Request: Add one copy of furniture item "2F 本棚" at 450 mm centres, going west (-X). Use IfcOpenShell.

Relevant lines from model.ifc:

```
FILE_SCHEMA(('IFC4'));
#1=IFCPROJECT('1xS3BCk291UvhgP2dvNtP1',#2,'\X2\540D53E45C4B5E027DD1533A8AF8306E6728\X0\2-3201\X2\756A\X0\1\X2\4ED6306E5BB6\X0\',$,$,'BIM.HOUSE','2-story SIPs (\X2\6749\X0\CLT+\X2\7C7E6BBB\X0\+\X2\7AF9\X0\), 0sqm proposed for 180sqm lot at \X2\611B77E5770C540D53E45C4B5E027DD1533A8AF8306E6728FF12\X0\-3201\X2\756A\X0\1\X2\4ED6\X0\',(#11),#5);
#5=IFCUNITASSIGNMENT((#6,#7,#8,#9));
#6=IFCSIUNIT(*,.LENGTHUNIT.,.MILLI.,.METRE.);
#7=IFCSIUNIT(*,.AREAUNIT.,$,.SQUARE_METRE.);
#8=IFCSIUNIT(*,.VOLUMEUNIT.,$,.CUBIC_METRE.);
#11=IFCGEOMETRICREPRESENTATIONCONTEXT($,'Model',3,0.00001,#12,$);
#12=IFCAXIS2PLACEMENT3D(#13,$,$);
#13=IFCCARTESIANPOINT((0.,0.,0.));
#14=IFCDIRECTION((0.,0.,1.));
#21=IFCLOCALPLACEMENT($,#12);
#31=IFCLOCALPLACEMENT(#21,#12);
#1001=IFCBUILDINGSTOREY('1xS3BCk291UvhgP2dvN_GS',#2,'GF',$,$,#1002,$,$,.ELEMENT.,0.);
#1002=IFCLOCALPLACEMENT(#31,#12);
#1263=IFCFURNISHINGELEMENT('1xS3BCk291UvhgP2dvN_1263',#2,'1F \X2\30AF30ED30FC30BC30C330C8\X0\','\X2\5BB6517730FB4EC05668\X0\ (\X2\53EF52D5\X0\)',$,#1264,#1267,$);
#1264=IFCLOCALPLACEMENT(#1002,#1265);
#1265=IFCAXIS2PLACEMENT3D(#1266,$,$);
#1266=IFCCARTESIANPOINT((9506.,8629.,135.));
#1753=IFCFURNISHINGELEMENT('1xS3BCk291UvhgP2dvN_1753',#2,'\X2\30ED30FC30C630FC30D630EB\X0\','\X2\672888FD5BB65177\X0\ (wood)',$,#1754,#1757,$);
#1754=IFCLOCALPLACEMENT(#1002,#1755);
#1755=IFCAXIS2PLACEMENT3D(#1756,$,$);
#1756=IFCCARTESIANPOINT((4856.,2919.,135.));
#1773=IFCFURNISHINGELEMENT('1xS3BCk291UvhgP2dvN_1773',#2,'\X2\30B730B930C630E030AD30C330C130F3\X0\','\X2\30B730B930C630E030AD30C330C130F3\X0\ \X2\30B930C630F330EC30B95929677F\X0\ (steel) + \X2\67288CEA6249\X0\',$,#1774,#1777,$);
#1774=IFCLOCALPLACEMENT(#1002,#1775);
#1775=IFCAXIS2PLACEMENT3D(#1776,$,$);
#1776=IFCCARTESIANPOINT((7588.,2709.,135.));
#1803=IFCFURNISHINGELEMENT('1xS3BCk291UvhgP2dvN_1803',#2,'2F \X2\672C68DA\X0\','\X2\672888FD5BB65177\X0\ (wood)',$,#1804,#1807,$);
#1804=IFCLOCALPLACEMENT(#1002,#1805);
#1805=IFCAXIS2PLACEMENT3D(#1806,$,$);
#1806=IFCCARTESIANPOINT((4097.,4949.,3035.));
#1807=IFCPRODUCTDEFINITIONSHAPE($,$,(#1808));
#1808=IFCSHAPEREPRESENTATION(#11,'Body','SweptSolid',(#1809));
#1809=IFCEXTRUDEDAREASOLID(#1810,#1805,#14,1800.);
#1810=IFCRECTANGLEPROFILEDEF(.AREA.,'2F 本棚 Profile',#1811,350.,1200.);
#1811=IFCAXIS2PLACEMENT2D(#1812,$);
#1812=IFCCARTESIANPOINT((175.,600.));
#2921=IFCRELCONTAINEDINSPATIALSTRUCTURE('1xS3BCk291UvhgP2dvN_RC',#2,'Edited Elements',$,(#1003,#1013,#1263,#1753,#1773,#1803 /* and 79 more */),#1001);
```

```python
import numpy as np
import ifcopenshell
import ifcopenshell.api.geometry
import ifcopenshell.api.root
import ifcopenshell.util.element
import ifcopenshell.util.placement

model = ifcopenshell.open("model.ifc")


def reuse_history(source, copy):
    """copy_class also copies each property set's owner history, people and application; keep the originals."""
    for rel in copy.IsDefinedBy:
        if rel.is_a("IfcRelDefinesByProperties") and (history := rel.RelatingPropertyDefinition.OwnerHistory):
            rel.RelatingPropertyDefinition.OwnerHistory = source.OwnerHistory
            ifcopenshell.util.element.remove_deep2(model, history)


source = model.by_guid("1xS3BCk291UvhgP2dvN_1803")
base = ifcopenshell.util.placement.get_local_placement(source.ObjectPlacement)
step = np.array([-1.0, 0.0, 0.0]) * 450.0

for i in range(1, 2):
    copy = ifcopenshell.api.root.copy_class(model, product=source)
    copy.Representation = ifcopenshell.util.element.copy_deep(
        model, source.Representation, exclude=["IfcGeometricRepresentationContext", "IfcRepresentationMap"]
    )
    reuse_history(source, copy)
    matrix = base.copy()
    matrix[:3, 3] += i * step
    print("added at", matrix[:3, 3].round(3) + 0.0)
    ifcopenshell.api.geometry.edit_object_placement(model, product=copy, matrix=matrix, is_si=False)

model.write("model_updated.ifc")
```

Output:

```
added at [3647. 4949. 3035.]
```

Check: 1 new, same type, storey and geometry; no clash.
